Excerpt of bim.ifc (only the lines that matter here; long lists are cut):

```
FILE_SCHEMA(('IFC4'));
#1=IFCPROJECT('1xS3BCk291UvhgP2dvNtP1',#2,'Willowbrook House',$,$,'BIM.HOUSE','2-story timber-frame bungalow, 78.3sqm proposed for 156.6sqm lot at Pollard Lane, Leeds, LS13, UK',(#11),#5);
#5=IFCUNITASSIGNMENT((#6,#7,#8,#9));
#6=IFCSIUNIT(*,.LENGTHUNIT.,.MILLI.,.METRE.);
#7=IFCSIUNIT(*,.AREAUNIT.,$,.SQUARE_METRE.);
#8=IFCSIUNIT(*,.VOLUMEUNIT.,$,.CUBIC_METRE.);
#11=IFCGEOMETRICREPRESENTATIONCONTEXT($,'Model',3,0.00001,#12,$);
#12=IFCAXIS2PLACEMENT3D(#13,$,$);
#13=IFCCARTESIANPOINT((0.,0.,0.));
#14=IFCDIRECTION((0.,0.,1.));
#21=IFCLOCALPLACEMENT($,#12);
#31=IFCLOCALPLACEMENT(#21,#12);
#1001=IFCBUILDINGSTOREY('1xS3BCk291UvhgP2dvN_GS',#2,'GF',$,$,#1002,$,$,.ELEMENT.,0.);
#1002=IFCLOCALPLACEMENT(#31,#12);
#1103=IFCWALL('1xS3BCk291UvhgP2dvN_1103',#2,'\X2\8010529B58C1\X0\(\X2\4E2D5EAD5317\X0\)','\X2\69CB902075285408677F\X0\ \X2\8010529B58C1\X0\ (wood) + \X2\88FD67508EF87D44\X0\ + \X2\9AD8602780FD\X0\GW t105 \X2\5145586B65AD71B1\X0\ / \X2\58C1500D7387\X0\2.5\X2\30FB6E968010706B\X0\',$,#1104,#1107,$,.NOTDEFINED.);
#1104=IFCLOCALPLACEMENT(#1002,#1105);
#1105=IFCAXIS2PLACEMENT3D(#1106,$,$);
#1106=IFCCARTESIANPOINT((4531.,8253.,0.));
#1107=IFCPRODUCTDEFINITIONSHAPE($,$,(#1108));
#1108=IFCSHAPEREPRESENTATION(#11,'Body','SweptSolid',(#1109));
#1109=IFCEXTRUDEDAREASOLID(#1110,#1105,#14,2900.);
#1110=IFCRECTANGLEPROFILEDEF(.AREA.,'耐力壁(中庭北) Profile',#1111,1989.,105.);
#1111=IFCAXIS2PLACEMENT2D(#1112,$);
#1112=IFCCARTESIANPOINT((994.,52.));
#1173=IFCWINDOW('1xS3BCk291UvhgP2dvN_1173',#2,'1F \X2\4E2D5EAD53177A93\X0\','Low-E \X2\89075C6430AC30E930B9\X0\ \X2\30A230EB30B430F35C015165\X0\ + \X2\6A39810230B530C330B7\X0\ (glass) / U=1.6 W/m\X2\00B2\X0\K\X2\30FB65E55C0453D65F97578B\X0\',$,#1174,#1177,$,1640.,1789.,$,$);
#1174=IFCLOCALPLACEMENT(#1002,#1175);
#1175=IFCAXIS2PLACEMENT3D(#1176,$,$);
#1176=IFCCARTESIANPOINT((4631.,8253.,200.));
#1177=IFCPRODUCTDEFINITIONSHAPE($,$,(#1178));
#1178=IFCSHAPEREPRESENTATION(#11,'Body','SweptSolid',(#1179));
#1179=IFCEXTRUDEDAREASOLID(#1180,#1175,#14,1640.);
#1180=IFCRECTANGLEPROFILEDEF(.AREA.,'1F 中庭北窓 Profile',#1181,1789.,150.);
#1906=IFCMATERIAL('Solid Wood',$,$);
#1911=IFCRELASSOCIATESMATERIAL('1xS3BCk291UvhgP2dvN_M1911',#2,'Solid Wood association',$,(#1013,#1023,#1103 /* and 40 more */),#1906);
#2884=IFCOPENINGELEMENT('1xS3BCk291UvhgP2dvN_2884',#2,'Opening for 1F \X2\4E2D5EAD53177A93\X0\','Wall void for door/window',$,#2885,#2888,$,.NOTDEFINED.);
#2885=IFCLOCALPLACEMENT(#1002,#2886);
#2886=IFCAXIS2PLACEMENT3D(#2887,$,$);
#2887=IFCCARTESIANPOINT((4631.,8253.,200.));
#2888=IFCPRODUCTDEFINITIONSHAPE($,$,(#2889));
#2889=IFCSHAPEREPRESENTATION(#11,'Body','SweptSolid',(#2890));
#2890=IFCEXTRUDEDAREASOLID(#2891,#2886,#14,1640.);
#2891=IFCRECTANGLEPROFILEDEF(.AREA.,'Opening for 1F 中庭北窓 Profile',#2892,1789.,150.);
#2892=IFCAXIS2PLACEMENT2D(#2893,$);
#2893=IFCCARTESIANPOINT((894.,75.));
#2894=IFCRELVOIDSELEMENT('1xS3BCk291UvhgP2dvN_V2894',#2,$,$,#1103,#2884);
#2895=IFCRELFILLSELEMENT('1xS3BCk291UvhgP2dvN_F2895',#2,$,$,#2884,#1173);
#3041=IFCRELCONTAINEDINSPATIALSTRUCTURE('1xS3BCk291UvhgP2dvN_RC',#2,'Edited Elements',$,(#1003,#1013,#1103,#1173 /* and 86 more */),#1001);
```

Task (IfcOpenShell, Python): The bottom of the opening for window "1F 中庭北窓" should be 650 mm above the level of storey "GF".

```python
import numpy as np
import ifcopenshell
import ifcopenshell.api.geometry
import ifcopenshell.geom
import ifcopenshell.util.element
import ifcopenshell.util.placement
import ifcopenshell.util.shape
import ifcopenshell.util.unit

model = ifcopenshell.open("bim.ifc")
unit_scale = ifcopenshell.util.unit.calculate_unit_scale(model)

window = model.by_guid("1xS3BCk291UvhgP2dvN_1173")
opening = window.FillsVoids[0].RelatingOpeningElement
storey = ifcopenshell.util.element.get_container(window, ifc_class="IfcBuildingStorey")
level = ifcopenshell.util.placement.get_local_placement(storey.ObjectPlacement)[2, 3]

# The opening's origin need not be at the sill, so measure its lowest point.
shape = ifcopenshell.geom.create_shape(ifcopenshell.geom.settings(), opening)
bottom = ifcopenshell.util.shape.get_shape_bottom_elevation(shape, shape.geometry) / unit_scale
dz = level + 0.65 / unit_scale - bottom

shift = np.array([0.0, 0.0, dz])
# The window is not placed relative to its opening, so move both.
for product in (opening, window):
    matrix = ifcopenshell.util.placement.get_local_placement(product.ObjectPlacement)
    matrix[:3, 3] += shift
    ifcopenshell.api.geometry.edit_object_placement(model, product=product, matrix=matrix, is_si=False)

print(f"moved by {dz * unit_scale:+.3f} m")

model.write("bim_v2.ifc")
```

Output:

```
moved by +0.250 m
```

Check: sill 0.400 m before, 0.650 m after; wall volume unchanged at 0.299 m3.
